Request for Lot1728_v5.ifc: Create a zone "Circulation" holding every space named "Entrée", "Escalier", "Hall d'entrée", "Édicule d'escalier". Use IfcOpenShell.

First a look at what the model holds.

```python
import ifcopenshell

model = ifcopenshell.open("Lot1728_v5.ifc")
print(model.schema)
seen = {}
for space in model.by_type("IfcSpace"):
    seen[space.LongName] = seen.get(space.LongName, 0) + 1
for name, count in sorted(seen.items(), key=str):
    print(count, "x", name)
print("zones:", [z.Name for z in model.by_type("IfcZone")][:20])
```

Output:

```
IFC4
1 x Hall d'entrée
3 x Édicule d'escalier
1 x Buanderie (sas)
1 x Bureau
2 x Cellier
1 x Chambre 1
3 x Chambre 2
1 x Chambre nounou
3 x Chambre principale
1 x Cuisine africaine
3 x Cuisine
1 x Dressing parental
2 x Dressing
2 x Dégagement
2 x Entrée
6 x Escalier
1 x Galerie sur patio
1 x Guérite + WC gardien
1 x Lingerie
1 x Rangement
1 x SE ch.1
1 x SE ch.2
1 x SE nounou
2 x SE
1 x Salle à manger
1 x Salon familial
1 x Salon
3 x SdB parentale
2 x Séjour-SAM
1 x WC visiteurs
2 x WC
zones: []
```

```python
import ifcopenshell
import ifcopenshell.api.group
import ifcopenshell.api.root

model = ifcopenshell.open("Lot1728_v5.ifc")

names = {"Entrée", "Escalier", "Hall d'entrée", "Édicule d'escalier"}
spaces = [s for s in model.by_type("IfcSpace") if s.LongName in names]

zone = ifcopenshell.api.root.create_entity(model, ifc_class="IfcZone", name="Circulation")
ifcopenshell.api.group.assign_group(model, products=spaces, group=zone)
print(len(spaces), "spaces in", zone.Name)

model.write("Lot1728_v5_rev.ifc")
```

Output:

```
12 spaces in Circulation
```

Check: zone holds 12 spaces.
